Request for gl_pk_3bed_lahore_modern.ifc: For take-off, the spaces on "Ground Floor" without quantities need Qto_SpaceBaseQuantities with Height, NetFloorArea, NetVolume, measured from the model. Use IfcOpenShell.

First a look at what the model holds.

```python
import ifcopenshell
import ifcopenshell.util.element
import ifcopenshell.util.unit

model = ifcopenshell.open("gl_pk_3bed_lahore_modern.ifc")
print(model.schema)
for unit_type in ("LENGTHUNIT", "AREAUNIT", "VOLUMEUNIT"):
    print(unit_type, ifcopenshell.util.unit.calculate_unit_scale(model, unit_type))
storey = next(s for s in model.by_type("IfcBuildingStorey") if s.Name == "Ground Floor")
spaces = [e for e in ifcopenshell.util.element.get_decomposition(storey) if e.is_a("IfcSpace")]
for e in sorted(spaces, key=lambda e: e.id()):
    print(e.id(), e.is_a(), e.Name, list(ifcopenshell.util.element.get_psets(e, qtos_only=True)), sep=" | ")
```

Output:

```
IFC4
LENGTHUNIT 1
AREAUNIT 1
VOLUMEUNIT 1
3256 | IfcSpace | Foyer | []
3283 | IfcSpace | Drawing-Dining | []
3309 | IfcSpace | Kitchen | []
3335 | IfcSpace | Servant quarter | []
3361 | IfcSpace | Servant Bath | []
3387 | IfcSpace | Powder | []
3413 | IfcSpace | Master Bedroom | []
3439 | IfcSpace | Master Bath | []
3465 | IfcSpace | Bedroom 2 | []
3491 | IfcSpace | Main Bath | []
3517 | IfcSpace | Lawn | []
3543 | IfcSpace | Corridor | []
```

```python
import ifcopenshell
import ifcopenshell.api.pset
import ifcopenshell.geom
import ifcopenshell.util.element
import ifcopenshell.util.shape
import ifcopenshell.util.unit

model = ifcopenshell.open("gl_pk_3bed_lahore_modern.ifc")
unit_scale = ifcopenshell.util.unit.calculate_unit_scale(model)
area_scale = ifcopenshell.util.unit.calculate_unit_scale(model, "AREAUNIT")
volume_scale = ifcopenshell.util.unit.calculate_unit_scale(model, "VOLUMEUNIT")
settings = ifcopenshell.geom.settings()

storey = next(s for s in model.by_type("IfcBuildingStorey") if s.Name == "Ground Floor")
spaces = [e for e in ifcopenshell.util.element.get_decomposition(storey) if e.is_a("IfcSpace")]

for e in sorted(spaces, key=lambda e: e.id()):
    if ifcopenshell.util.element.get_psets(e, qtos_only=True, should_inherit=False):
        continue
    # Geometry comes back in metres, in the element's own axes.
    shape = ifcopenshell.geom.create_shape(settings, e)
    values = {
        "Height": ifcopenshell.util.shape.get_z(shape.geometry) / unit_scale,
        "NetFloorArea": ifcopenshell.util.shape.get_footprint_area(shape.geometry) / area_scale,
        "NetVolume": ifcopenshell.util.shape.get_volume(shape.geometry) / volume_scale,
    }
    qto = ifcopenshell.api.pset.add_qto(model, product=e, name="Qto_SpaceBaseQuantities")
    ifcopenshell.api.pset.edit_qto(model, qto=qto, properties=values)
    print(e.id(), {k: round(v, 3) for k, v in values.items()})

model.write("gl_pk_3bed_lahore_modern-out.ifc")
```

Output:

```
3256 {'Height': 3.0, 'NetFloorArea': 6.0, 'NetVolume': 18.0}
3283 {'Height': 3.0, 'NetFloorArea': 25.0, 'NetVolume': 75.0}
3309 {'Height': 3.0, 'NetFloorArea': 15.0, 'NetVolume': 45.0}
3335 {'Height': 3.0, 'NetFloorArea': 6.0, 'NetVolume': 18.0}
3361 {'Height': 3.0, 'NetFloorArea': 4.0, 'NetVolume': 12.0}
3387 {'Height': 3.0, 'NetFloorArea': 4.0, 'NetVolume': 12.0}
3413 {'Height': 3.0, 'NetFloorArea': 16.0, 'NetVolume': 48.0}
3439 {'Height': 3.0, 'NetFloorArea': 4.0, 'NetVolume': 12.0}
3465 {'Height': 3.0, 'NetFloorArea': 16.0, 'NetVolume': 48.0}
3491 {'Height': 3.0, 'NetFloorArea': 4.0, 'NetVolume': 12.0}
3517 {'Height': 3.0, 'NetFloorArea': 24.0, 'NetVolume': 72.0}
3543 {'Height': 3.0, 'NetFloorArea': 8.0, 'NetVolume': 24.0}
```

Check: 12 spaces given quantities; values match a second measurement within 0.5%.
